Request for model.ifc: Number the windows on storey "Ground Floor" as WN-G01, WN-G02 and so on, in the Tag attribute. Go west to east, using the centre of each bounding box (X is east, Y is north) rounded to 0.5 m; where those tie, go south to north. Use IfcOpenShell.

First a look at what the model holds.

```python
import ifcopenshell
import ifcopenshell.util.element
import ifcopenshell.util.placement

model = ifcopenshell.open("model.ifc")
print(model.schema)
storey = next(s for s in model.by_type("IfcBuildingStorey") if s.Name == "Ground Floor")
windows = [e for e in ifcopenshell.util.element.get_decomposition(storey) if e.is_a("IfcWindow")]
for e in sorted(windows, key=lambda e: e.id()):
    origin = ifcopenshell.util.placement.get_local_placement(e.ObjectPlacement)[:3, 3]
    print(e.id(), e.Tag, e.Name, origin.round(2) + 0.0, sep=" | ")
```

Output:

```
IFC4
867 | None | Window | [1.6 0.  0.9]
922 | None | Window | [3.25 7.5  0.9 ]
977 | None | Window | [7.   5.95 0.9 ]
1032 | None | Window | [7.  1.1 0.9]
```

```python
import ifcopenshell
import ifcopenshell.geom
import ifcopenshell.util.element
import ifcopenshell.util.shape

model = ifcopenshell.open("model.ifc")
settings = ifcopenshell.geom.settings()
settings.set("use-world-coords", True)


def centre(element):
    shape = ifcopenshell.geom.create_shape(settings, element)
    return ifcopenshell.util.shape.get_bbox_centroid(shape.geometry)


storey = next(s for s in model.by_type("IfcBuildingStorey") if s.Name == "Ground Floor")
windows = [e for e in ifcopenshell.util.element.get_decomposition(storey) if e.is_a("IfcWindow")]

# Insertion points can sit at a corner or the storey origin, so sort by the geometry (in metres).
centres = {e: centre(e) for e in windows}
windows.sort(key=lambda e: (round(centres[e][0] / 0.5), centres[e][1]))

for i, e in enumerate(windows, start=1):
    number = f"WN-G{i:02d}"
    e.Tag = number
    print(e.id(), number)

model.write("model_edited.ifc")
```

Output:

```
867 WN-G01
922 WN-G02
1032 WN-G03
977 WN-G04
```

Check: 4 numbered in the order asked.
